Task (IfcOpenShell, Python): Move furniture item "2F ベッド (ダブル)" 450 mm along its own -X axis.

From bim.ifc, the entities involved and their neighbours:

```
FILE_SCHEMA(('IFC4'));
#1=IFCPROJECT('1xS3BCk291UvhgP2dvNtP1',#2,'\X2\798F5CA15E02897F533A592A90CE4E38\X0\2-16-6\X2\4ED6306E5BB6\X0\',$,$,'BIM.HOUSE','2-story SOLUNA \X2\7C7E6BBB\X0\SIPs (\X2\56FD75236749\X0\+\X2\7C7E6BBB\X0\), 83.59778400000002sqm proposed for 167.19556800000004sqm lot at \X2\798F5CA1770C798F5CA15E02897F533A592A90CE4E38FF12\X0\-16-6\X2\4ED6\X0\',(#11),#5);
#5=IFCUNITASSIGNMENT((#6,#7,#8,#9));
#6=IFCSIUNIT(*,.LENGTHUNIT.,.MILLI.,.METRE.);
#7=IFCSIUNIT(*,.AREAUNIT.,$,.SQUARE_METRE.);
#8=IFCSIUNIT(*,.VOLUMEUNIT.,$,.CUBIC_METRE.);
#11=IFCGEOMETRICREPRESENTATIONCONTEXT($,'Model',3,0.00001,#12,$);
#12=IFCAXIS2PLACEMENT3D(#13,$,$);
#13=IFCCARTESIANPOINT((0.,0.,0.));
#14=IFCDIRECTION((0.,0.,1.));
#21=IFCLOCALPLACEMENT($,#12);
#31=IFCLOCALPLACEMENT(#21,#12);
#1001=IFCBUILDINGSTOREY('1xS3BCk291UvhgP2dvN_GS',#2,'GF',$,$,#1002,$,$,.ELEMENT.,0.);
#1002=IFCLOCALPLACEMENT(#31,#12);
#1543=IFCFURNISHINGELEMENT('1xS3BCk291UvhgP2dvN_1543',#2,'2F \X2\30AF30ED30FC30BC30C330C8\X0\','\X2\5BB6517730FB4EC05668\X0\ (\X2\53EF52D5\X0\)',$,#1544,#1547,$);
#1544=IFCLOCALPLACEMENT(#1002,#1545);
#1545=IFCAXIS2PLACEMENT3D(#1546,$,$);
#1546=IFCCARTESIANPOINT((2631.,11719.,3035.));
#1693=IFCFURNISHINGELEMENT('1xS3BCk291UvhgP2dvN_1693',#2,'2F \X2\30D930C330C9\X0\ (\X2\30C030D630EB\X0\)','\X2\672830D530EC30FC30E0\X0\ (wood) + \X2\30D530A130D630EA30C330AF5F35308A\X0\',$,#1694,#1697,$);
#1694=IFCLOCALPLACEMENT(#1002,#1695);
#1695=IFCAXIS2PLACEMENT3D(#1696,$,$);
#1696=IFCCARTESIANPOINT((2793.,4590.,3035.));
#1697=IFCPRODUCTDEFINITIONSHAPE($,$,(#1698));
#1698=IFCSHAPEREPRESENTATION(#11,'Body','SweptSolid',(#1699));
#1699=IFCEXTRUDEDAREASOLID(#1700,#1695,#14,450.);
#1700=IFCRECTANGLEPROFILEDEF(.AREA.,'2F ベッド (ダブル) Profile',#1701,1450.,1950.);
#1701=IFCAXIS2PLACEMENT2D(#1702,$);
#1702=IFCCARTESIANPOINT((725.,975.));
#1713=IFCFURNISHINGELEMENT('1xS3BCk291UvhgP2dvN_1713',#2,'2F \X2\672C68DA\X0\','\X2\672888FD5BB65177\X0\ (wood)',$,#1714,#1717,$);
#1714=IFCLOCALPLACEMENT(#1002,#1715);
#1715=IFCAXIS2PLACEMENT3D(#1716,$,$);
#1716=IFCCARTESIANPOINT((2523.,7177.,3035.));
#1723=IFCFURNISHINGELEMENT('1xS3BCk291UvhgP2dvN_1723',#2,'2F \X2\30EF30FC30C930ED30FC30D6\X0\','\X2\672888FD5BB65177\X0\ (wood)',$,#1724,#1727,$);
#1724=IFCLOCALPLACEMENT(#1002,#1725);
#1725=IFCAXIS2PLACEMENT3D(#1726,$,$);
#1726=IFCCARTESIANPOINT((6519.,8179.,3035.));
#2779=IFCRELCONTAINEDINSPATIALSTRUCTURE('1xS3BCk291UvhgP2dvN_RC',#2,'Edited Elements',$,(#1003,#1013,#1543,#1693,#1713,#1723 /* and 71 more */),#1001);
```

```python
import ifcopenshell
import ifcopenshell.api.geometry
import ifcopenshell.util.placement

model = ifcopenshell.open("bim.ifc")

item = model.by_id(1693)
matrix = ifcopenshell.util.placement.get_local_placement(item.ObjectPlacement)
matrix[:3, 3] -= matrix[:3, 0] * 450.0
ifcopenshell.api.geometry.edit_object_placement(model, product=item, matrix=matrix, is_si=False)

print(ifcopenshell.util.placement.get_local_placement(item.ObjectPlacement).round(3) + 0.0)

model.write("bim_edited.ifc")
```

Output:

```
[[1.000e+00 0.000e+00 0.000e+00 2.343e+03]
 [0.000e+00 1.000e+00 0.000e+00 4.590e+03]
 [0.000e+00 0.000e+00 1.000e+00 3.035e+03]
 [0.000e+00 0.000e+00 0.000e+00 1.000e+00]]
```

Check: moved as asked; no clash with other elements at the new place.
